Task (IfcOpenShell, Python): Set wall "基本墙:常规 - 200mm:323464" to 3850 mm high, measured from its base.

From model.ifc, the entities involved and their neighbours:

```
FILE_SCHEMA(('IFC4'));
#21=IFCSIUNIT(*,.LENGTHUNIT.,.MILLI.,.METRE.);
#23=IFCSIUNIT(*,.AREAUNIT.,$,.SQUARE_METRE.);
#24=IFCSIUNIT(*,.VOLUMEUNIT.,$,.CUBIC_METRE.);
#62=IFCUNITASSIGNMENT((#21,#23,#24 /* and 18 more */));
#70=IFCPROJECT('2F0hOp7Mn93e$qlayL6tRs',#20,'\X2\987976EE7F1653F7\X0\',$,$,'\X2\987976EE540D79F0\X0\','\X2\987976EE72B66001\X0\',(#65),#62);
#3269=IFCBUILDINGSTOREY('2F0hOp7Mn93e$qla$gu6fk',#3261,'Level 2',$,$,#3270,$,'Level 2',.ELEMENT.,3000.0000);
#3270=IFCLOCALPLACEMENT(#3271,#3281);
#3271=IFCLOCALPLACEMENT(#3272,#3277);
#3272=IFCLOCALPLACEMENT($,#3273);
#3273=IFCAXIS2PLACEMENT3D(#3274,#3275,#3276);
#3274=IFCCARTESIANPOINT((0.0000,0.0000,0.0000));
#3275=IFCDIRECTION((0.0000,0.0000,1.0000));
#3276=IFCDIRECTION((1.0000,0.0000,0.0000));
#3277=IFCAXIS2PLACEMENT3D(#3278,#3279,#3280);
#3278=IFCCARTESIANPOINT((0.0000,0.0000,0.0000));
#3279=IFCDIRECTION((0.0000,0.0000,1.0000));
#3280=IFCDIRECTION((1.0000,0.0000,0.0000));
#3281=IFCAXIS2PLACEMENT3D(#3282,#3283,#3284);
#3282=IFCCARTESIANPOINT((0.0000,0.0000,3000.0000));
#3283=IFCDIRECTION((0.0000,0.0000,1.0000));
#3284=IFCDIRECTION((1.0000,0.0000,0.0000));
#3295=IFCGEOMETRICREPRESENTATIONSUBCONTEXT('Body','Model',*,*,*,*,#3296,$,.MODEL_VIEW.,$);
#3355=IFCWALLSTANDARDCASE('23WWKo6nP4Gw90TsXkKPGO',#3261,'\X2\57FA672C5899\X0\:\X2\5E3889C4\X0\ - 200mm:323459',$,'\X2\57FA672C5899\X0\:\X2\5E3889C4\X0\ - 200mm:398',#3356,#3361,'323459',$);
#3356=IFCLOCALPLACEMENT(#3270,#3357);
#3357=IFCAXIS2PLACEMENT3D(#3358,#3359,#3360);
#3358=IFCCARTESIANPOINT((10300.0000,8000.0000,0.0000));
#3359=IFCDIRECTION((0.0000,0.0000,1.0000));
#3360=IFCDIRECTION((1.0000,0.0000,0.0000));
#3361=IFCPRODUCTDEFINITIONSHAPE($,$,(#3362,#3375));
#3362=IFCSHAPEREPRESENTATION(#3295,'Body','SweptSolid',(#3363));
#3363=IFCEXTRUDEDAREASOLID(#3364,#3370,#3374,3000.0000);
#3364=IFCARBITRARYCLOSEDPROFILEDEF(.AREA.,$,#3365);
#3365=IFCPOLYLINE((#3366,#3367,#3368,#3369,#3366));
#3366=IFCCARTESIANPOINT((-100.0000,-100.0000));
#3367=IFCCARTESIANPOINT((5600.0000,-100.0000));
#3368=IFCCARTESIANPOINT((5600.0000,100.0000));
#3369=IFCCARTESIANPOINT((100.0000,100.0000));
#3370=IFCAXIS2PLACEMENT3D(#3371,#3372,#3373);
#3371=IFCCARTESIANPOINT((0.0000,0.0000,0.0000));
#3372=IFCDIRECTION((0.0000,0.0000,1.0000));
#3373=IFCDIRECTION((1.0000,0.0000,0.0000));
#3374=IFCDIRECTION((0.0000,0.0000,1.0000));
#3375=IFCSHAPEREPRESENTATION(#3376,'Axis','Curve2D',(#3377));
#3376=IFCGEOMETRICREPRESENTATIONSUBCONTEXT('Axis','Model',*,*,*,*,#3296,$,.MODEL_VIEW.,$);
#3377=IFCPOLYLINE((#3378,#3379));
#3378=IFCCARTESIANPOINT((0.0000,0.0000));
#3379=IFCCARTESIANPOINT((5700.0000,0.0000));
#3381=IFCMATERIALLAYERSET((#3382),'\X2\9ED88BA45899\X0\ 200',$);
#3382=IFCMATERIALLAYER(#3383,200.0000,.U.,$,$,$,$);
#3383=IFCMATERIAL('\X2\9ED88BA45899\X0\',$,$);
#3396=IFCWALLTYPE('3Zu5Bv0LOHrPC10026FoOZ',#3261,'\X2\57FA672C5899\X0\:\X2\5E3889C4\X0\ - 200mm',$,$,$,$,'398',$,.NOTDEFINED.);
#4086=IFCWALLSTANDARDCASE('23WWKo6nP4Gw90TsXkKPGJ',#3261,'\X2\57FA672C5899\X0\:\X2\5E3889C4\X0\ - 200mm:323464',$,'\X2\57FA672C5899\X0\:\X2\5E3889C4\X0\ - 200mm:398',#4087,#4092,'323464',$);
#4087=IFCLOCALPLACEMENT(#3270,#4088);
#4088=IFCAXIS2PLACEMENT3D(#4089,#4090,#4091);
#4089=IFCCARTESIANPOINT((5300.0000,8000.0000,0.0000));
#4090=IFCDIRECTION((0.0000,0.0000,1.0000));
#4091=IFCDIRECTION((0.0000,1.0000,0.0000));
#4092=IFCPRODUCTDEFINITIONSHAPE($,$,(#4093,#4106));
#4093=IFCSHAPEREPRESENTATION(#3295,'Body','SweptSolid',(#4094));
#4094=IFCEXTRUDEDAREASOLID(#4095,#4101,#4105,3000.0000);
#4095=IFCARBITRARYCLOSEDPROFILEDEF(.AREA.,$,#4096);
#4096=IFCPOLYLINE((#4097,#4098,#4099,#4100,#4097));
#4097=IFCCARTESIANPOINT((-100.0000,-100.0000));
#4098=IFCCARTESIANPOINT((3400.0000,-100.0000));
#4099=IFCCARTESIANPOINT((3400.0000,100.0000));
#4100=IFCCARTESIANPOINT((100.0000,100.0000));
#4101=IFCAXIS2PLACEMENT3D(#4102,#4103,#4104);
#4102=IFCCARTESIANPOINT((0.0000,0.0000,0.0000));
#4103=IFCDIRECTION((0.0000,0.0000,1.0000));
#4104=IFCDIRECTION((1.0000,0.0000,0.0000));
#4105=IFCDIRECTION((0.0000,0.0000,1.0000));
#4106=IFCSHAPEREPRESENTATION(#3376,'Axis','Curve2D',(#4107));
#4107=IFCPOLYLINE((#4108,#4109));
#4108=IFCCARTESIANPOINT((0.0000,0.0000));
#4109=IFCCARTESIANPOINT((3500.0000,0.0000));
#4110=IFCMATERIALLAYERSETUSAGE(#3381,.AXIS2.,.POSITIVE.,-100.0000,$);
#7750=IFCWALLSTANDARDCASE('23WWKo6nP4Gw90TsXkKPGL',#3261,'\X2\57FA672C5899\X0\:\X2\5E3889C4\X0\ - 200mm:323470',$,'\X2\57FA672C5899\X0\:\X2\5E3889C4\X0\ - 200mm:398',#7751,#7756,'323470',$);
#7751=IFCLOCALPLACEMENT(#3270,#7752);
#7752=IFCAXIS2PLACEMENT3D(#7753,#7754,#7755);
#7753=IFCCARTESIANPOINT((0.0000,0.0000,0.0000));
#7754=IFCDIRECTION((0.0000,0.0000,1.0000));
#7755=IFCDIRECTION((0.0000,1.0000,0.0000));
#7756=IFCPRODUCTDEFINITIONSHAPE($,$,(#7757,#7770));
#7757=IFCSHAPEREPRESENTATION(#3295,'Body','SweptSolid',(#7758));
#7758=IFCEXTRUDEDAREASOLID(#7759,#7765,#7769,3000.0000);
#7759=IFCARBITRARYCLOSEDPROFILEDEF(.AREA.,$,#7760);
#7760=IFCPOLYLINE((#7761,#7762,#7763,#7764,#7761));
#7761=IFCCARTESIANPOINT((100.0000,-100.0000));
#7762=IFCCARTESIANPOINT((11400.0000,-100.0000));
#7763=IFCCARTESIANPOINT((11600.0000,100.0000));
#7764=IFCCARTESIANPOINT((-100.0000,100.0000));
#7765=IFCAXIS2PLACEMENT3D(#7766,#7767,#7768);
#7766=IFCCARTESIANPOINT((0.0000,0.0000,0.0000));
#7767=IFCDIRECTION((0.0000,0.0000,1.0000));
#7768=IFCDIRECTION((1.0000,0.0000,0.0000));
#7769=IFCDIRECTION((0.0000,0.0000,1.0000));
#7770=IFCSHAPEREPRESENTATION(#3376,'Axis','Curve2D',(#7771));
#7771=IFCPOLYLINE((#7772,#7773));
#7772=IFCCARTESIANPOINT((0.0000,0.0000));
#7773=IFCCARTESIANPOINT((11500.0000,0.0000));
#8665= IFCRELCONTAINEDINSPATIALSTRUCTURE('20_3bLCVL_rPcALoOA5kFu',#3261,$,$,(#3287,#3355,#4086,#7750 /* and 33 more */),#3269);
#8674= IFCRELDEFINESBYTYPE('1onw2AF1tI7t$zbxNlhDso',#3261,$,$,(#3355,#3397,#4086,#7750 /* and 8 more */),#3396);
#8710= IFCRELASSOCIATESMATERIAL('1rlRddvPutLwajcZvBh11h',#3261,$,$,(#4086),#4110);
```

```python
import ifcopenshell
import ifcopenshell.geom
import ifcopenshell.util.representation
import ifcopenshell.util.shape
import ifcopenshell.util.unit

model = ifcopenshell.open("model.ifc")
unit_scale = ifcopenshell.util.unit.calculate_unit_scale(model)
settings = ifcopenshell.geom.settings()


def volume(element):
    """Net volume in cubic metres, openings subtracted."""
    shape = ifcopenshell.geom.create_shape(settings, element)
    return ifcopenshell.util.shape.get_volume(shape.geometry)


wall = model.by_guid("23WWKo6nP4Gw90TsXkKPGJ")
before = volume(wall)

body = ifcopenshell.util.representation.get_representation(wall, "Model", "Body")
solid = body.Items[0]
old_height = solid.Depth
solid.Depth = 3.85 / unit_scale
after = volume(wall)

print(f"height {old_height:g} -> {solid.Depth:g}, volume {before:.3f} -> {after:.3f} m3")

model.write("model_edited.ifc")
```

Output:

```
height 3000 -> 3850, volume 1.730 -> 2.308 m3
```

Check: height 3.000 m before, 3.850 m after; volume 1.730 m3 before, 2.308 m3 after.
